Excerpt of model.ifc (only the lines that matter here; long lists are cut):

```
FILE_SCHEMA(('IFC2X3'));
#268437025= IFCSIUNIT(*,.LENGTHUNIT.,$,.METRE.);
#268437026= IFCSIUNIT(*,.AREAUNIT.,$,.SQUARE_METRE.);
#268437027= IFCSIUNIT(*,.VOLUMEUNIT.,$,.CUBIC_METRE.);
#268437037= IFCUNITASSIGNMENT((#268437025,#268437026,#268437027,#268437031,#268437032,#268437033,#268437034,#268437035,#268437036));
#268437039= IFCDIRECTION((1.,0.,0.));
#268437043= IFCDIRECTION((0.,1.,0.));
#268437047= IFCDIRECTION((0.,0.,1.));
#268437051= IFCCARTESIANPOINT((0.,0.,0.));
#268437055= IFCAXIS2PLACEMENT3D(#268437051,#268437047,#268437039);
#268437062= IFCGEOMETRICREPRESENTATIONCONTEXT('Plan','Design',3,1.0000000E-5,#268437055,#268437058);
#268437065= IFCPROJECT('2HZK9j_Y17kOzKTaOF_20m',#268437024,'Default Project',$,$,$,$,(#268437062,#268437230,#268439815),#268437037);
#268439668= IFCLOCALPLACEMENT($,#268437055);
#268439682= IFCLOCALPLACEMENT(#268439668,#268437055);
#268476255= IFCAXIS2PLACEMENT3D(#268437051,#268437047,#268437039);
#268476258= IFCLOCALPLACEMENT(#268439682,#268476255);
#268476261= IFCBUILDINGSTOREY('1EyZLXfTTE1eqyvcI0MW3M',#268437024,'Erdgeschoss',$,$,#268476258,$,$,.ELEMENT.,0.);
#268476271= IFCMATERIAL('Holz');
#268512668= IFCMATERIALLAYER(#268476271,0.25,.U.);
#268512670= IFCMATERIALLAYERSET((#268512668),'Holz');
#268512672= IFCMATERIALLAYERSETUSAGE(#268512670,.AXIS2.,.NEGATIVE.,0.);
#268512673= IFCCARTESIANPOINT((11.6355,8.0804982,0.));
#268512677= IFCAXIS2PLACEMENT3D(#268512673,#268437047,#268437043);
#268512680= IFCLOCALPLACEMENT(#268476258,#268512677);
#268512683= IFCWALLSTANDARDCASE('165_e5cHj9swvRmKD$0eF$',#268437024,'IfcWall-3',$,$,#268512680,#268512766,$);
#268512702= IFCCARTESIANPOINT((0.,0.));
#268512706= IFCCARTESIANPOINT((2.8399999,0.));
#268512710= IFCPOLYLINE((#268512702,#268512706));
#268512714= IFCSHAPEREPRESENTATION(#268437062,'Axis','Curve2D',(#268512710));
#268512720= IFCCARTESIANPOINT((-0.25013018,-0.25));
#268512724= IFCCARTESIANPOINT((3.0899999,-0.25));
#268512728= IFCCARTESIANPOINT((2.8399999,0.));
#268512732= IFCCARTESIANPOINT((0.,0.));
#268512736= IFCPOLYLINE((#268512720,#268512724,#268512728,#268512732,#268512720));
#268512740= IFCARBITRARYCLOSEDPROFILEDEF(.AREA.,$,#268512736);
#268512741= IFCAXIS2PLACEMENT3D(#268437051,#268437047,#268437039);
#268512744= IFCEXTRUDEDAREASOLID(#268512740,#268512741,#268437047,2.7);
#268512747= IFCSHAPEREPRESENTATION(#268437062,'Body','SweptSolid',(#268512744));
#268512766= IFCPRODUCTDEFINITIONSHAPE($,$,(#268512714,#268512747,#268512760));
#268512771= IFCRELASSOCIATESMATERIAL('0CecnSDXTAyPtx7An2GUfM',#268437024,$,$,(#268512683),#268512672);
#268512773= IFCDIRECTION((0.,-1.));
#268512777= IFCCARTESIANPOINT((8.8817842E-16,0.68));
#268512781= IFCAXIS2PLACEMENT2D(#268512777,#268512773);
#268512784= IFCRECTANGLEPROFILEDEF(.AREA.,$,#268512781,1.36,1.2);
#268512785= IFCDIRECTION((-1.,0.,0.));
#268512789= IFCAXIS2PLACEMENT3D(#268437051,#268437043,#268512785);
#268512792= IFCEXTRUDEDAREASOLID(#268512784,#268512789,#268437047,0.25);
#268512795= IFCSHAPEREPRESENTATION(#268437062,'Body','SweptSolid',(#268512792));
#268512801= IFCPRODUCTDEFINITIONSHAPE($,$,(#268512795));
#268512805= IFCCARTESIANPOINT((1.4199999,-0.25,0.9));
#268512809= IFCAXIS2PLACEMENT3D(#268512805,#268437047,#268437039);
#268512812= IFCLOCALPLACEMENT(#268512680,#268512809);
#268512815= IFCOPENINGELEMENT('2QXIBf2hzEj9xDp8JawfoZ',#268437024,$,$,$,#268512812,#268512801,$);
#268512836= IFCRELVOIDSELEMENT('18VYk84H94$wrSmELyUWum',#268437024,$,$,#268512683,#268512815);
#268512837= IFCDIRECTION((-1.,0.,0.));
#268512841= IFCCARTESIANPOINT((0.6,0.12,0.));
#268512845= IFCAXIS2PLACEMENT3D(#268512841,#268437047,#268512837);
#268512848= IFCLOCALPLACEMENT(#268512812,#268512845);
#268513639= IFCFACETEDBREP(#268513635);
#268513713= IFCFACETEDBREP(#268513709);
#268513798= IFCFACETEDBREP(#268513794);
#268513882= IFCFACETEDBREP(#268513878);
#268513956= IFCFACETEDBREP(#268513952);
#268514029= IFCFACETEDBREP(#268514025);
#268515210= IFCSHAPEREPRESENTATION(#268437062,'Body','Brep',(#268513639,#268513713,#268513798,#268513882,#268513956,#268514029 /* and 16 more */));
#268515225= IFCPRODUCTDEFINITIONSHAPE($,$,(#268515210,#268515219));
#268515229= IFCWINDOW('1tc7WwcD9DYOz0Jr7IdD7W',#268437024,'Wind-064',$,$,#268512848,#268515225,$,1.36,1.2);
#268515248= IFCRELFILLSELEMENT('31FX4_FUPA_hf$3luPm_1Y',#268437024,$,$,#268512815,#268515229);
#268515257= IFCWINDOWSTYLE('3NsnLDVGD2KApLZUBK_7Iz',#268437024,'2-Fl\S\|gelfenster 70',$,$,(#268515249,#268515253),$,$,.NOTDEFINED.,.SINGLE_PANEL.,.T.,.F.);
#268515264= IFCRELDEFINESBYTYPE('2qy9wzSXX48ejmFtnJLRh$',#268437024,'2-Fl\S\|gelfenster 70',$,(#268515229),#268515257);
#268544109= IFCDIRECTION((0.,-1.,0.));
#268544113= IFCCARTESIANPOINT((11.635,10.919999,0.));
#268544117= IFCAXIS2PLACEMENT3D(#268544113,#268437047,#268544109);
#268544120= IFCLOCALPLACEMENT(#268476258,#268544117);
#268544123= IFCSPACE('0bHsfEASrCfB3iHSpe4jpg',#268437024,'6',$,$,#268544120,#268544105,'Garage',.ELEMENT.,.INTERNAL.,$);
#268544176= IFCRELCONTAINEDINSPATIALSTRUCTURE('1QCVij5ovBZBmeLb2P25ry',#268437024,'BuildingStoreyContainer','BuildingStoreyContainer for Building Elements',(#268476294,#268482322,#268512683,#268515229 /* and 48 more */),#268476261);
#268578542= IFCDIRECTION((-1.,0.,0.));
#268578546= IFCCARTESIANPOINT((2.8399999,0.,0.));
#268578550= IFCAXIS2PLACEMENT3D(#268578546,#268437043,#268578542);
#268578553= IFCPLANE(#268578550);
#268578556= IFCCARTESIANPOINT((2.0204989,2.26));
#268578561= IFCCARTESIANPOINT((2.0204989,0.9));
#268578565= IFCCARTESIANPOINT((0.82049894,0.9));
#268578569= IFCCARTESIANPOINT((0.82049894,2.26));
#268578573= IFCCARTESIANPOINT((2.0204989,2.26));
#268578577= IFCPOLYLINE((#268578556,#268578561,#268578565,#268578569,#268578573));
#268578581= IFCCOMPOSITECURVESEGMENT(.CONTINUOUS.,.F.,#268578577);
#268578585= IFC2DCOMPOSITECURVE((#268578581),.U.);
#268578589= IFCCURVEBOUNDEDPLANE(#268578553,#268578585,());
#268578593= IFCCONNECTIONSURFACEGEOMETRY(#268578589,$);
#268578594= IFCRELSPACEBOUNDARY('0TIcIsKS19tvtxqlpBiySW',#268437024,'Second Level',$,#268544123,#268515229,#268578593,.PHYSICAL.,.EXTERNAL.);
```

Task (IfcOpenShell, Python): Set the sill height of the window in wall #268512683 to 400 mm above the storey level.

```python
import numpy as np
import ifcopenshell
import ifcopenshell.api.geometry
import ifcopenshell.geom
import ifcopenshell.util.element
import ifcopenshell.util.placement
import ifcopenshell.util.shape
import ifcopenshell.util.unit

model = ifcopenshell.open("model.ifc")
unit_scale = ifcopenshell.util.unit.calculate_unit_scale(model)

window = model.by_id(268515229)
opening = window.FillsVoids[0].RelatingOpeningElement
storey = ifcopenshell.util.element.get_container(window, ifc_class="IfcBuildingStorey")
level = ifcopenshell.util.placement.get_local_placement(storey.ObjectPlacement)[2, 3]

# The opening's origin need not be at the sill, so measure its lowest point.
shape = ifcopenshell.geom.create_shape(ifcopenshell.geom.settings(), opening)
bottom = ifcopenshell.util.shape.get_shape_bottom_elevation(shape, shape.geometry) / unit_scale
dz = level + 0.4 / unit_scale - bottom

shift = np.array([0.0, 0.0, dz])
# The window is placed relative to its opening, so it follows when the opening moves.
matrix = ifcopenshell.util.placement.get_local_placement(opening.ObjectPlacement)
matrix[:3, 3] += shift
ifcopenshell.api.geometry.edit_object_placement(
    model, product=opening, matrix=matrix, is_si=False, should_transform_children=True
)

# Space boundary surfaces are stored in each space's coordinates; move them too.
for rel in window.ProvidesBoundaries:
    if not rel.ConnectionGeometry:
        continue
    surface = rel.ConnectionGeometry.SurfaceOnRelatingElement.BasisSurface
    space_matrix = ifcopenshell.util.placement.get_local_placement(rel.RelatingSpace.ObjectPlacement)
    point = np.array(surface.Position.Location.Coordinates) + space_matrix[:3, :3].T @ shift
    surface.Position = model.createIfcAxis2Placement3D(
        model.createIfcCartesianPoint(point.tolist()), surface.Position.Axis, surface.Position.RefDirection
    )

print(f"moved by {dz * unit_scale:+.3f} m")

model.write("model_updated.ifc")
```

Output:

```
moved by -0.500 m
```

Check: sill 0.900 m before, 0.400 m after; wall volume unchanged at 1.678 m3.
